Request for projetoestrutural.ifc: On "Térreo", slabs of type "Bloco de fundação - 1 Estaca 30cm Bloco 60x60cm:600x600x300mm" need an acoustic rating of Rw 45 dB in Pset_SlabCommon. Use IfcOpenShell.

First a look at what the model holds.

```python
import ifcopenshell
import ifcopenshell.util.element

model = ifcopenshell.open("projetoestrutural.ifc")
print(model.schema)
storey = next(s for s in model.by_type("IfcBuildingStorey") if s.Name == "Térreo")
slabs = [e for e in ifcopenshell.util.element.get_decomposition(storey) if e.is_a("IfcSlab")]
seen = {}
for e in slabs:
    element_type = ifcopenshell.util.element.get_type(e)
    key = (element_type.Name if element_type != e and element_type else None, ifcopenshell.util.element.get_pset(e, "Pset_SlabCommon", "AcousticRating"))
    seen[key] = seen.get(key, 0) + 1
for (name, value), count in sorted(seen.items(), key=str):
    print(count, "x", name, "|", value)
```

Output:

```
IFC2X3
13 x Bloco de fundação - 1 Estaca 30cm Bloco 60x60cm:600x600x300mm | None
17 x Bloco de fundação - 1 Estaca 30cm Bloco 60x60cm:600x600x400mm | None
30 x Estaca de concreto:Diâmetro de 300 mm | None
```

```python
import ifcopenshell
import ifcopenshell.api.pset
import ifcopenshell.util.element

model = ifcopenshell.open("projetoestrutural.ifc")

storey = next(s for s in model.by_type("IfcBuildingStorey") if s.Name == "Térreo")
slabs = [e for e in ifcopenshell.util.element.get_decomposition(storey) if e.is_a("IfcSlab")]

count = 0
for e in slabs:
    element_type = ifcopenshell.util.element.get_type(e)
    if element_type in (None, e) or element_type.Name != "Bloco de fundação - 1 Estaca 30cm Bloco 60x60cm:600x600x300mm":
        continue
    # add_pset returns the element's existing set when there is one.
    pset = ifcopenshell.api.pset.add_pset(model, product=e, name="Pset_SlabCommon")
    ifcopenshell.api.pset.edit_pset(model, pset=pset, properties={"AcousticRating": "Rw 45 dB"})
    count += 1

print(count, "slabs updated")

model.write("projetoestrutural_updated.ifc")
```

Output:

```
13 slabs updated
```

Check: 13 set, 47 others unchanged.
